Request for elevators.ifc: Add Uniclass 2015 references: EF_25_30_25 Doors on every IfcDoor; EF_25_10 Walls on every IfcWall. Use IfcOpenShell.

First a look at what the model holds.

```python
import ifcopenshell

model = ifcopenshell.open("elevators.ifc")
print(model.schema)
print("classifications:", [c.Name for c in model.by_type("IfcClassification")])
for ifc_class in ("IfcDoor", "IfcRoof", "IfcStair", "IfcWall", "IfcWindow"):
    print(ifc_class, len(model.by_type(ifc_class)))
```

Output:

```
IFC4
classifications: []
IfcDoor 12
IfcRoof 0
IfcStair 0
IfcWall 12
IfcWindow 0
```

```python
import ifcopenshell
import ifcopenshell.api.classification

model = ifcopenshell.open("elevators.ifc")

system = ifcopenshell.api.classification.add_classification(model, classification="Uniclass 2015")

codes = {
    "IfcDoor": ("EF_25_30_25", "Doors"),
    "IfcWall": ("EF_25_10", "Walls"),
}
for ifc_class, (code, name) in codes.items():
    products = model.by_type(ifc_class)
    ifcopenshell.api.classification.add_reference(
        model, products=products, classification=system, identification=code, name=name
    )
    print(code, len(products))

model.write("elevators_edited.ifc")
```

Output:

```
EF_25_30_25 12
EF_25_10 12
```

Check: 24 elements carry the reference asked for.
